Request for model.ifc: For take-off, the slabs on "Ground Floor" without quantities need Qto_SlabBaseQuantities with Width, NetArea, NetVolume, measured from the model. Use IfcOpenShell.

First a look at what the model holds.

```python
import ifcopenshell
import ifcopenshell.util.element
import ifcopenshell.util.unit

model = ifcopenshell.open("model.ifc")
print(model.schema)
for unit_type in ("LENGTHUNIT", "AREAUNIT", "VOLUMEUNIT"):
    print(unit_type, ifcopenshell.util.unit.calculate_unit_scale(model, unit_type))
storey = next(s for s in model.by_type("IfcBuildingStorey") if s.Name == "Ground Floor")
slabs = [e for e in ifcopenshell.util.element.get_decomposition(storey) if e.is_a("IfcSlab")]
for e in sorted(slabs, key=lambda e: e.id()):
    print(e.id(), e.is_a(), e.Name, list(ifcopenshell.util.element.get_psets(e, qtos_only=True)), sep=" | ")
```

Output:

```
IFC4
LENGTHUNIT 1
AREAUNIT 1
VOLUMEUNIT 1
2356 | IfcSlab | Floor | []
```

```python
import ifcopenshell
import ifcopenshell.api.pset
import ifcopenshell.geom
import ifcopenshell.util.element
import ifcopenshell.util.shape
import ifcopenshell.util.unit

model = ifcopenshell.open("model.ifc")
unit_scale = ifcopenshell.util.unit.calculate_unit_scale(model)
area_scale = ifcopenshell.util.unit.calculate_unit_scale(model, "AREAUNIT")
volume_scale = ifcopenshell.util.unit.calculate_unit_scale(model, "VOLUMEUNIT")
settings = ifcopenshell.geom.settings()

storey = next(s for s in model.by_type("IfcBuildingStorey") if s.Name == "Ground Floor")
slabs = [e for e in ifcopenshell.util.element.get_decomposition(storey) if e.is_a("IfcSlab")]

for e in sorted(slabs, key=lambda e: e.id()):
    if ifcopenshell.util.element.get_psets(e, qtos_only=True, should_inherit=False):
        continue
    # Geometry comes back in metres, in the element's own axes.
    shape = ifcopenshell.geom.create_shape(settings, e)
    values = {
        "Width": ifcopenshell.util.shape.get_z(shape.geometry) / unit_scale,
        "NetArea": ifcopenshell.util.shape.get_footprint_area(shape.geometry) / area_scale,
        "NetVolume": ifcopenshell.util.shape.get_volume(shape.geometry) / volume_scale,
    }
    qto = ifcopenshell.api.pset.add_qto(model, product=e, name="Qto_SlabBaseQuantities")
    ifcopenshell.api.pset.edit_qto(model, qto=qto, properties=values)
    print(e.id(), {k: round(v, 3) for k, v in values.items()})

model.write("model-out.ifc")
```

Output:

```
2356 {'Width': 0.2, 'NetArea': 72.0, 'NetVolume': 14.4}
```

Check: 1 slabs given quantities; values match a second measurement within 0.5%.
